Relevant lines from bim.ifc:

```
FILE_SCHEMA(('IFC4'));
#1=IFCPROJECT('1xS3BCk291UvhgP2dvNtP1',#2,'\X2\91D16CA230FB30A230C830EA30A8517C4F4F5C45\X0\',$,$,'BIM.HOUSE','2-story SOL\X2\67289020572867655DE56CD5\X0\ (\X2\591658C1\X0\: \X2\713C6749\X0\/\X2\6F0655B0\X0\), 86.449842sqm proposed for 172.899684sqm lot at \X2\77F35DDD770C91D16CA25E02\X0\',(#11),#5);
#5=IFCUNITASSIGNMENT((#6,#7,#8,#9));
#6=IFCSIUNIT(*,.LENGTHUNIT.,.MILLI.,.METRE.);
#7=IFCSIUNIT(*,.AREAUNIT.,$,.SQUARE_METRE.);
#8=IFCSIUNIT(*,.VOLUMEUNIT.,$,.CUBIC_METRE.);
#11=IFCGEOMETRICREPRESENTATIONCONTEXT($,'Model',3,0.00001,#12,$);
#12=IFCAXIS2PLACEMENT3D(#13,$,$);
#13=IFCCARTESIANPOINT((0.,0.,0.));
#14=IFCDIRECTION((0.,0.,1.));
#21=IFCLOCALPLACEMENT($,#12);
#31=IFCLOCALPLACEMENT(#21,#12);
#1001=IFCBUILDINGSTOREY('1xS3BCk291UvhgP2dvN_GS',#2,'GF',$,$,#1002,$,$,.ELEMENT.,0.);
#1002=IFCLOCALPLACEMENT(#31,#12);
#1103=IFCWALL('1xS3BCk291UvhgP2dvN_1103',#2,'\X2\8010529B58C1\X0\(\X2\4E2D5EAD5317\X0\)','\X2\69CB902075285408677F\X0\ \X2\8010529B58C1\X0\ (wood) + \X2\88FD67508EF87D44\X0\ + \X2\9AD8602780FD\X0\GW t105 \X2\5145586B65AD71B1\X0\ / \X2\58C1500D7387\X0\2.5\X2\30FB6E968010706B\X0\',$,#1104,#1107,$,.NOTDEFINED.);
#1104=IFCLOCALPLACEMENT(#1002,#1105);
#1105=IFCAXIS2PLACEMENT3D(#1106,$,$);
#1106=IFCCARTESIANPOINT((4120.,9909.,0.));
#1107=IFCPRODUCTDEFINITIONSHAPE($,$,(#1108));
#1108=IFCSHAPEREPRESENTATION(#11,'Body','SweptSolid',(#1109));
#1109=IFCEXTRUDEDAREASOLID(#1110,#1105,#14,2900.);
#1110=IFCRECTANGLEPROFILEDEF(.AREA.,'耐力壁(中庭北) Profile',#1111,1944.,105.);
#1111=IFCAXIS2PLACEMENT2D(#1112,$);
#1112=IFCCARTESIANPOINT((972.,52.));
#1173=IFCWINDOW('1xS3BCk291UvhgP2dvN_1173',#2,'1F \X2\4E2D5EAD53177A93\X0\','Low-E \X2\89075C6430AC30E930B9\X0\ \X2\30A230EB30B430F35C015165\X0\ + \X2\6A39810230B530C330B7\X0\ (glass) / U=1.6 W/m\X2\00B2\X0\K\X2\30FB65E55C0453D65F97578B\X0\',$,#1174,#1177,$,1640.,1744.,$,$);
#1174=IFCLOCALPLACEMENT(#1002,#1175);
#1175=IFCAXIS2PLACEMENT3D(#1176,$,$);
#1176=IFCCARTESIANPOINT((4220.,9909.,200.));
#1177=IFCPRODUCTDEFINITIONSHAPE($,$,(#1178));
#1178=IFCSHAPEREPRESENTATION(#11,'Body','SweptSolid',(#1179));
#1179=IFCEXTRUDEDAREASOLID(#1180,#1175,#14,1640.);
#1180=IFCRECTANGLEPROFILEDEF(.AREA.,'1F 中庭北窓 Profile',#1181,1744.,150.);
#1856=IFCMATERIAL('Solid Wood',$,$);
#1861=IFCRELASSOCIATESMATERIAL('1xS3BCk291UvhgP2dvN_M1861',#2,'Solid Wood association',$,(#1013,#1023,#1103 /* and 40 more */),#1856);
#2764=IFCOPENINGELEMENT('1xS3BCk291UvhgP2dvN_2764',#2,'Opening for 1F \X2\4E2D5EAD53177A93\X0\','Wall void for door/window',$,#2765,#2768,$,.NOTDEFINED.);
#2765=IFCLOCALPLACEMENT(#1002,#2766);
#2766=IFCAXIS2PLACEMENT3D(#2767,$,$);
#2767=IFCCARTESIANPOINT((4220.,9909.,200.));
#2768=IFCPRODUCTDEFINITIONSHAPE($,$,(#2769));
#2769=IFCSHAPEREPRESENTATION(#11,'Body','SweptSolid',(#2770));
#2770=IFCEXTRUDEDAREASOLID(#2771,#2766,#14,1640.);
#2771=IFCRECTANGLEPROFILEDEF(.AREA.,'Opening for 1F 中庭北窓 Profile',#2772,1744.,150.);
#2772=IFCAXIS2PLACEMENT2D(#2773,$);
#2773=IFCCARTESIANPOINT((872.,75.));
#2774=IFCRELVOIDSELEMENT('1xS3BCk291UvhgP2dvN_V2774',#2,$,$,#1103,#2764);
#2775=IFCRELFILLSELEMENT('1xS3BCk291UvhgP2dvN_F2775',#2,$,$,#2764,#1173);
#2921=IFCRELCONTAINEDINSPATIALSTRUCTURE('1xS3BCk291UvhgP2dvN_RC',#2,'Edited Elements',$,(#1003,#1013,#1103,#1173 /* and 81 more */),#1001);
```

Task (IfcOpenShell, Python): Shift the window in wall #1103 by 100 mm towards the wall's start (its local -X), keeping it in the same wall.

```python
import ifcopenshell
import ifcopenshell.api.geometry
import ifcopenshell.util.placement

model = ifcopenshell.open("bim.ifc")

window = model.by_guid("1xS3BCk291UvhgP2dvN_1173")
opening = window.FillsVoids[0].RelatingOpeningElement
wall = opening.VoidsElements[0].RelatingBuildingElement

wall_matrix = ifcopenshell.util.placement.get_local_placement(wall.ObjectPlacement)
shift = wall_matrix[:3, 0] * -100.0
before = ifcopenshell.util.placement.get_local_placement(window.ObjectPlacement)[:3, 3].copy()

# The window is not placed relative to its opening, so move both.
for product in (opening, window):
    matrix = ifcopenshell.util.placement.get_local_placement(product.ObjectPlacement)
    matrix[:3, 3] += shift
    ifcopenshell.api.geometry.edit_object_placement(model, product=product, matrix=matrix, is_si=False)

after = ifcopenshell.util.placement.get_local_placement(window.ObjectPlacement)[:3, 3]
print("window moved by", (after - before).round(3) + 0.0)

model.write("bim_v2.ifc")
```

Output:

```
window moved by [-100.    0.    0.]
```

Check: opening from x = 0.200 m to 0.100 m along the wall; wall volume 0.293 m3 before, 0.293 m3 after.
